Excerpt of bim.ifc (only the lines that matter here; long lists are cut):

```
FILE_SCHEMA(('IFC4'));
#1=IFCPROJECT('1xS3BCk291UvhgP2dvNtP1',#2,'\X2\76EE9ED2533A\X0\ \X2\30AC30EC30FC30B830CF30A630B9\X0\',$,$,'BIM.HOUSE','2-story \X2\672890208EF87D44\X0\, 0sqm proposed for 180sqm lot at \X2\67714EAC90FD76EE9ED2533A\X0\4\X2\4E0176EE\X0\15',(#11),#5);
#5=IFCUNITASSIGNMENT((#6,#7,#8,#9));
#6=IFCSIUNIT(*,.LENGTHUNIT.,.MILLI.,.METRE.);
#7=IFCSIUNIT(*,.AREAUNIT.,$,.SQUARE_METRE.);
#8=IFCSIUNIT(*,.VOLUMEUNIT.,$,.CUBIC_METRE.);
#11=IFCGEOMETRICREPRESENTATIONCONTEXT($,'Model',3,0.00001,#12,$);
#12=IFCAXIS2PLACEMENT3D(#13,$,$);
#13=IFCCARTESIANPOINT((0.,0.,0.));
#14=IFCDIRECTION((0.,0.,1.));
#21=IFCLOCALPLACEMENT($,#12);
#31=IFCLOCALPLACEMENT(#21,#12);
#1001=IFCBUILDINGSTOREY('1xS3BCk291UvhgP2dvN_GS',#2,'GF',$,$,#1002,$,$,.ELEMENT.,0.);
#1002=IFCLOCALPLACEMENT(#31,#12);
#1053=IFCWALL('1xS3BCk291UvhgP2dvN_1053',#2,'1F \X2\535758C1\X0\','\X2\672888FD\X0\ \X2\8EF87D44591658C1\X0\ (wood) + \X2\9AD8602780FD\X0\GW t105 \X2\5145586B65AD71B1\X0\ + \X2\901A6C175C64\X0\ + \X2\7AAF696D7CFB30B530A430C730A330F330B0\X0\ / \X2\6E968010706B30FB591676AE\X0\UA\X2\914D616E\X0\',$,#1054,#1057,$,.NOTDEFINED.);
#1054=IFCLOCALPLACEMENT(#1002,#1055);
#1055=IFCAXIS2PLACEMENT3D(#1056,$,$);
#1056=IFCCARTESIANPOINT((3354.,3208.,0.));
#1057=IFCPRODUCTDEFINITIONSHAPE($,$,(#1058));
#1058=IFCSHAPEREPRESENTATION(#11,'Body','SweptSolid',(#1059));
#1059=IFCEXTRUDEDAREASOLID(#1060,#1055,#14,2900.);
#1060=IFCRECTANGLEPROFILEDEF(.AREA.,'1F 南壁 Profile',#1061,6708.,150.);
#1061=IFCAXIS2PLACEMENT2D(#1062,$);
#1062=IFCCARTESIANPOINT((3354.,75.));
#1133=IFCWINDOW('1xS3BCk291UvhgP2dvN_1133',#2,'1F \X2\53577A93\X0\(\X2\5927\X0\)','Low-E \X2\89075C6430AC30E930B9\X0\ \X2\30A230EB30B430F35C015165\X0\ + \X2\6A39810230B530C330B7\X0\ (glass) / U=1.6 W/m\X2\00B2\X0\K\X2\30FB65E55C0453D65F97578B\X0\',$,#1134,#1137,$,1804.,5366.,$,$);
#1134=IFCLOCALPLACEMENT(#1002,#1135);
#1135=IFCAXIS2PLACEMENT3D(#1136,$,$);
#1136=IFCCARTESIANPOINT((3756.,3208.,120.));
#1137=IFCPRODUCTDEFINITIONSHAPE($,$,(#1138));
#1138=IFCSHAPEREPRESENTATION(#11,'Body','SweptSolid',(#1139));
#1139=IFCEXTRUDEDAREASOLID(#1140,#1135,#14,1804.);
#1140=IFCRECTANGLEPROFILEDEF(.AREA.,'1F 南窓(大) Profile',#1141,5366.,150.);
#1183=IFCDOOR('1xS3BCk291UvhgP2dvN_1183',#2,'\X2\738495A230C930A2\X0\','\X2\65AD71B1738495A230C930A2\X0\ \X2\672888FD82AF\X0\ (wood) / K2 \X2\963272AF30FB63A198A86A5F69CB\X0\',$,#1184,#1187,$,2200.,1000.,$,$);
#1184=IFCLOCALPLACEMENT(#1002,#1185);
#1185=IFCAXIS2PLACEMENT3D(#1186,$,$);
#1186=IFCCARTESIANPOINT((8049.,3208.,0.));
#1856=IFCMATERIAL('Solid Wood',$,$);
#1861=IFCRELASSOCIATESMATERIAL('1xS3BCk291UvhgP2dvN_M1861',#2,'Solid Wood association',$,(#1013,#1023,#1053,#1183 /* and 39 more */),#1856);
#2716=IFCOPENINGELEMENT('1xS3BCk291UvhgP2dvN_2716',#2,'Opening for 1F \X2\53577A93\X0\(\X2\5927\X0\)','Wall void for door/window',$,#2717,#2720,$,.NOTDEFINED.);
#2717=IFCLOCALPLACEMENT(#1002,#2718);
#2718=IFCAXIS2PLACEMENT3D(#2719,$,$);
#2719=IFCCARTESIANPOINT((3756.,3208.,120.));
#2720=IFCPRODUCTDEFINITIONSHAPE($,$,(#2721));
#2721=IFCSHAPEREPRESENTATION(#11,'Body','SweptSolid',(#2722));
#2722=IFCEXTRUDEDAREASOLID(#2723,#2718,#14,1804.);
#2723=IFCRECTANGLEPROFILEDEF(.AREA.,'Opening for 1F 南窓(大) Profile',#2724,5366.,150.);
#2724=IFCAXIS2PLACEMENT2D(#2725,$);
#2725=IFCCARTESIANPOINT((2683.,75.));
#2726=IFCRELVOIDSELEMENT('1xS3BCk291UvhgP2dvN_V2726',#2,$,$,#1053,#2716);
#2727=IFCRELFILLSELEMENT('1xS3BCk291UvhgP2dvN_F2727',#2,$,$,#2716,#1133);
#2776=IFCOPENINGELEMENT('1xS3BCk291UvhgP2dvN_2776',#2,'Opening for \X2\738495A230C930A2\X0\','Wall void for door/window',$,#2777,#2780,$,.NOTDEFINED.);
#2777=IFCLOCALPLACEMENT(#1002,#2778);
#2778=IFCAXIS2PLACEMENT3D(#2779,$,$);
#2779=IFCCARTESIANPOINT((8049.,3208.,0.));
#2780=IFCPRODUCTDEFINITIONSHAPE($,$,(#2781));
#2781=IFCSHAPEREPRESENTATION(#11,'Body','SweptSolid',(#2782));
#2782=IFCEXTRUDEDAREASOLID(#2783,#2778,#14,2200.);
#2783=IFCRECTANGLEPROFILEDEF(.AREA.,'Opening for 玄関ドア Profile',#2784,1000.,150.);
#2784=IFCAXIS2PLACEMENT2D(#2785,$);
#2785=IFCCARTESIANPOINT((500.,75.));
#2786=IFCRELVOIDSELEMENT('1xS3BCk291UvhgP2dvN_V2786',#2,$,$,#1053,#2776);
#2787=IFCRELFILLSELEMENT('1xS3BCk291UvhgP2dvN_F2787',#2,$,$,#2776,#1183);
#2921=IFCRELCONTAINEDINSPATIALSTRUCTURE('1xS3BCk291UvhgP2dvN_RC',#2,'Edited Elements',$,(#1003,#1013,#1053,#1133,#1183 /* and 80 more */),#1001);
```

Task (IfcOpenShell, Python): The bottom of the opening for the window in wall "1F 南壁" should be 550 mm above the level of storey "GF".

```python
import numpy as np
import ifcopenshell
import ifcopenshell.api.geometry
import ifcopenshell.geom
import ifcopenshell.util.element
import ifcopenshell.util.placement
import ifcopenshell.util.shape
import ifcopenshell.util.unit

model = ifcopenshell.open("bim.ifc")
unit_scale = ifcopenshell.util.unit.calculate_unit_scale(model)

window = model.by_guid("1xS3BCk291UvhgP2dvN_1133")
opening = window.FillsVoids[0].RelatingOpeningElement
storey = ifcopenshell.util.element.get_container(window, ifc_class="IfcBuildingStorey")
level = ifcopenshell.util.placement.get_local_placement(storey.ObjectPlacement)[2, 3]

# The opening's origin need not be at the sill, so measure its lowest point.
shape = ifcopenshell.geom.create_shape(ifcopenshell.geom.settings(), opening)
bottom = ifcopenshell.util.shape.get_shape_bottom_elevation(shape, shape.geometry) / unit_scale
dz = level + 550.0 - bottom

shift = np.array([0.0, 0.0, dz])
# The window is not placed relative to its opening, so move both.
for product in (opening, window):
    matrix = ifcopenshell.util.placement.get_local_placement(product.ObjectPlacement)
    matrix[:3, 3] += shift
    ifcopenshell.api.geometry.edit_object_placement(model, product=product, matrix=matrix, is_si=False)

print(f"moved by {dz * unit_scale:+.3f} m")

model.write("bim_rev.ifc")
```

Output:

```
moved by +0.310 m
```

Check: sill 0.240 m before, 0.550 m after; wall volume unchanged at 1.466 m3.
